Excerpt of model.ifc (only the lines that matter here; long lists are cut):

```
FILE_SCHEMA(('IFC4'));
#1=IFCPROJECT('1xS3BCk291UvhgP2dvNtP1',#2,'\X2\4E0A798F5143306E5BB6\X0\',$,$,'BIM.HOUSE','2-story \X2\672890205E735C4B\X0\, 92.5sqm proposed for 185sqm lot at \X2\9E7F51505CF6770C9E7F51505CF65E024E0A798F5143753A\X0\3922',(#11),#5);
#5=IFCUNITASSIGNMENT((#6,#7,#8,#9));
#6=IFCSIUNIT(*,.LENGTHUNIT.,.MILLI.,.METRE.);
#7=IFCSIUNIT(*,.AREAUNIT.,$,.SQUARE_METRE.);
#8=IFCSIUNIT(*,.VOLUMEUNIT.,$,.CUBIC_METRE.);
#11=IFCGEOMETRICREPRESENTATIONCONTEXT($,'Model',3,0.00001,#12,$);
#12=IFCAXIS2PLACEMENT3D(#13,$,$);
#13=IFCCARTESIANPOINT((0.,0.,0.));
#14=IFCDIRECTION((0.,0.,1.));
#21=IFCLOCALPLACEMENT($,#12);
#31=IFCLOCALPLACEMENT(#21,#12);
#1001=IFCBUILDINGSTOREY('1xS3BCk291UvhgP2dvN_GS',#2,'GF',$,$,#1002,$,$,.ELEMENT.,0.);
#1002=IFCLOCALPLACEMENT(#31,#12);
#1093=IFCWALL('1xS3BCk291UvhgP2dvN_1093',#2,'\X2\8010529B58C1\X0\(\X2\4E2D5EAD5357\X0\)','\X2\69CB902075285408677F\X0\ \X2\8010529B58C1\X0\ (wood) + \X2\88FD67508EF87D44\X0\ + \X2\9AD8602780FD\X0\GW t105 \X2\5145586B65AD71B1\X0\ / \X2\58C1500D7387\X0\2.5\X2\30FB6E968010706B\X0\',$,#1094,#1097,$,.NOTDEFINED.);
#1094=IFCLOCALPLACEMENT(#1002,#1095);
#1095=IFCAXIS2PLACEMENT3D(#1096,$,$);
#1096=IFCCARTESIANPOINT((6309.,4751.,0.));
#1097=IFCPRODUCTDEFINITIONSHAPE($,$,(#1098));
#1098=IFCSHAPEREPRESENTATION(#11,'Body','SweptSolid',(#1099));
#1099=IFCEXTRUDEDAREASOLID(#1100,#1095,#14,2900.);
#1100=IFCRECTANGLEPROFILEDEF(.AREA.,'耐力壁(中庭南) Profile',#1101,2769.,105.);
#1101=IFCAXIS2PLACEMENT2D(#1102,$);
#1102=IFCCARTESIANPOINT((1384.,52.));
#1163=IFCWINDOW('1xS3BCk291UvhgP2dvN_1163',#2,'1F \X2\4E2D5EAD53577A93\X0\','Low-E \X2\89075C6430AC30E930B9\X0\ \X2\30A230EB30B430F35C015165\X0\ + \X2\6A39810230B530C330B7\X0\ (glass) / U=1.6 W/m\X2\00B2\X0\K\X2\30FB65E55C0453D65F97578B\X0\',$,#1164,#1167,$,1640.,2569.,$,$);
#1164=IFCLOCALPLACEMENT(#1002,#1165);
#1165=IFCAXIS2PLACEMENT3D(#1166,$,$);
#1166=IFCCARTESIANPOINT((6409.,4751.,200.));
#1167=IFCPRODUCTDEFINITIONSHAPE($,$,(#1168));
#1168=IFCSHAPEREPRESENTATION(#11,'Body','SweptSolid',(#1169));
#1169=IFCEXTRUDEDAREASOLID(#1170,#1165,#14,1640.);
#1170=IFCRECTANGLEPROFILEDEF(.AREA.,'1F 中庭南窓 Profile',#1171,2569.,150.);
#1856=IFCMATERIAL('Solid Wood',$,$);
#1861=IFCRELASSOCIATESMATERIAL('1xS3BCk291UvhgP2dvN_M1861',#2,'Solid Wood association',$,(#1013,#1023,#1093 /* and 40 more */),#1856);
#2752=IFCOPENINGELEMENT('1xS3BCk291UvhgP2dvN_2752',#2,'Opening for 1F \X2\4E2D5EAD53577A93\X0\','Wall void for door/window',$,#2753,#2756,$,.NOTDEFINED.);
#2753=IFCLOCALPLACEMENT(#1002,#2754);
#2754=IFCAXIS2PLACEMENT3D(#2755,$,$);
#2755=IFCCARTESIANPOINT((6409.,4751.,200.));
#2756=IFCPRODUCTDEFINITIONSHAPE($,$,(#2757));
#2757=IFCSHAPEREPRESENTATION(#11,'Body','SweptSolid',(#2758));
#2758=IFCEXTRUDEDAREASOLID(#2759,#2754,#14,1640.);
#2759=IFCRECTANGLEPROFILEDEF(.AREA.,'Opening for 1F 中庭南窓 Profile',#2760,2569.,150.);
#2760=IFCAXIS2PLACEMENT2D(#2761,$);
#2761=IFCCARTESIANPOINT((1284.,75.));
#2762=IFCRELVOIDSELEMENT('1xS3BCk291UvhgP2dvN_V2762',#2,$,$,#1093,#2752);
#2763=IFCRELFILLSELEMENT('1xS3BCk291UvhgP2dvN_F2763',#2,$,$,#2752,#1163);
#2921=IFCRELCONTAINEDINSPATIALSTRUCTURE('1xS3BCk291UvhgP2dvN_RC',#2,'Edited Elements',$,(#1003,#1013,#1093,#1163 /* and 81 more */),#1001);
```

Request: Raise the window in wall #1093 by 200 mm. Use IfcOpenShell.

```python
import numpy as np
import ifcopenshell
import ifcopenshell.api.geometry
import ifcopenshell.util.placement
import ifcopenshell.util.unit

model = ifcopenshell.open("model.ifc")
unit_scale = ifcopenshell.util.unit.calculate_unit_scale(model)

window = model.by_id(1163)
opening = window.FillsVoids[0].RelatingOpeningElement
dz = 0.2 / unit_scale

shift = np.array([0.0, 0.0, dz])
# The window is not placed relative to its opening, so move both.
for product in (opening, window):
    matrix = ifcopenshell.util.placement.get_local_placement(product.ObjectPlacement)
    matrix[:3, 3] += shift
    ifcopenshell.api.geometry.edit_object_placement(model, product=product, matrix=matrix, is_si=False)

print(f"moved by {dz * unit_scale:+.3f} m")

model.write("model-out.ifc")
```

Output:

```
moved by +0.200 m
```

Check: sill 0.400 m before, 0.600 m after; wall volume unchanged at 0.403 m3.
